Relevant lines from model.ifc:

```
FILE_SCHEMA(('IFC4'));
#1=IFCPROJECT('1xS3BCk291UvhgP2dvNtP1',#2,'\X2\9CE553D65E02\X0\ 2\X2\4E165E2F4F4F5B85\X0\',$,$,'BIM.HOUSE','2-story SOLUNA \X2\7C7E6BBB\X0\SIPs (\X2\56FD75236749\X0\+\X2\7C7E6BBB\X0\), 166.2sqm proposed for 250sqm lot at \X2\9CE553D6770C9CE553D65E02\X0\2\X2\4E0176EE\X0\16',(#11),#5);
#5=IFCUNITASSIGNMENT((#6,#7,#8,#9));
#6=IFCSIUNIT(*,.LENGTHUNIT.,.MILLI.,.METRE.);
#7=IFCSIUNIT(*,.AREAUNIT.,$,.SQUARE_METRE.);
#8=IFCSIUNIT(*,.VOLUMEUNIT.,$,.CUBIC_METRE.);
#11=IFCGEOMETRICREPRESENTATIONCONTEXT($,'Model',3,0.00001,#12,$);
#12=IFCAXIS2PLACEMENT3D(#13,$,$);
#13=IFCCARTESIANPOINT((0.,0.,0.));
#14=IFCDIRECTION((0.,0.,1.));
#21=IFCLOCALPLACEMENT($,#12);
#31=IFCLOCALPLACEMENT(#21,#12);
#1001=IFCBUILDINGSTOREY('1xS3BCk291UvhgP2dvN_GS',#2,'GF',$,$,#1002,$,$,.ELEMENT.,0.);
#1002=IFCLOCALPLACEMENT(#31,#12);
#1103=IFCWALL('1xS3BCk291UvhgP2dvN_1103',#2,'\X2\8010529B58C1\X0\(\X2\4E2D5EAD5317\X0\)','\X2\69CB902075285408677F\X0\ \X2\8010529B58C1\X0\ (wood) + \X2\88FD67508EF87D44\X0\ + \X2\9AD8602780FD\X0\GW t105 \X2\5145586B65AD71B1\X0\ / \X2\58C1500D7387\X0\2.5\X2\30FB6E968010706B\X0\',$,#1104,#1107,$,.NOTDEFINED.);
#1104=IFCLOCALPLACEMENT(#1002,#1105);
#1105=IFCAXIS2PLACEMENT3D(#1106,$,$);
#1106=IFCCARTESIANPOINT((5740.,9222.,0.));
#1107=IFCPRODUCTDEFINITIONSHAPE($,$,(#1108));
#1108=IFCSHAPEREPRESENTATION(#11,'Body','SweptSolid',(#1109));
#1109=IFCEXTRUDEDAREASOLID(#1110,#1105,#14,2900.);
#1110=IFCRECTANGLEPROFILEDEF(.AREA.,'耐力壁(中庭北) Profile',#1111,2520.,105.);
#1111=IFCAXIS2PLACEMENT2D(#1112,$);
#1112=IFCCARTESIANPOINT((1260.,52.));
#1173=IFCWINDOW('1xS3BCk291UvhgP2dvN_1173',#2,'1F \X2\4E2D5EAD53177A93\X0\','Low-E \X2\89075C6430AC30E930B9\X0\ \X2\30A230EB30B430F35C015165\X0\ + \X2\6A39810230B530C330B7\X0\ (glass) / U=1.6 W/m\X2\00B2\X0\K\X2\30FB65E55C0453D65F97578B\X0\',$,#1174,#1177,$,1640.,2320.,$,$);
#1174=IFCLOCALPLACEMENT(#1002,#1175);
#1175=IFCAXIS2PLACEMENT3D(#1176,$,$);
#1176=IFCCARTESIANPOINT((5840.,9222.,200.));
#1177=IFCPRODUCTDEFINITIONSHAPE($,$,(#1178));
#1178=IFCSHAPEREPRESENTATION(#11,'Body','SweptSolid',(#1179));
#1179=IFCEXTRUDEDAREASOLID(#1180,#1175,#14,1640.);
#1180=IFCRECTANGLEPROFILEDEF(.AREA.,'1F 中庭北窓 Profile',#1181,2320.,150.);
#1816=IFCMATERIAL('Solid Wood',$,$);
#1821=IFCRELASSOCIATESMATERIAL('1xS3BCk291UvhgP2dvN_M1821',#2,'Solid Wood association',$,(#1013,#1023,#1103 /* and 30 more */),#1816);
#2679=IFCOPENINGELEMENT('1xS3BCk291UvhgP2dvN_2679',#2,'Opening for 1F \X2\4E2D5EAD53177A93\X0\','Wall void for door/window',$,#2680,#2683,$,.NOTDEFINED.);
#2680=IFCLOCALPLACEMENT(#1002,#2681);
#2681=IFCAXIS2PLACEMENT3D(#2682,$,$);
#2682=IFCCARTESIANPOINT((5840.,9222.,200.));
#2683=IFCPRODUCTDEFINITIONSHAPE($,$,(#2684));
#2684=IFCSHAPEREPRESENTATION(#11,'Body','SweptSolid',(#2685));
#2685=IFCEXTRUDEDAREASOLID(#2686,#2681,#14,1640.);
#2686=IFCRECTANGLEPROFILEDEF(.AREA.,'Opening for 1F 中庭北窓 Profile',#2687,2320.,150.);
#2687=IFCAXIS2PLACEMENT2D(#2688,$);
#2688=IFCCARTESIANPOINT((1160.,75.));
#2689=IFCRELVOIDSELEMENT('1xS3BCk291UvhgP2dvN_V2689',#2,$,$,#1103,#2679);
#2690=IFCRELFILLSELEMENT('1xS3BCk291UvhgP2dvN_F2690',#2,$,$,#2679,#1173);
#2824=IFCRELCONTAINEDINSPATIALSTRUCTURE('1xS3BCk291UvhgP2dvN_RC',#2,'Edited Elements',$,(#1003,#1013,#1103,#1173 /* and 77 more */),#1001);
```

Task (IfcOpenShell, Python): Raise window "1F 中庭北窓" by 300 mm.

```python
import numpy as np
import ifcopenshell
import ifcopenshell.api.geometry
import ifcopenshell.util.placement
import ifcopenshell.util.unit

model = ifcopenshell.open("model.ifc")
unit_scale = ifcopenshell.util.unit.calculate_unit_scale(model)

window = model.by_guid("1xS3BCk291UvhgP2dvN_1173")
opening = window.FillsVoids[0].RelatingOpeningElement
dz = 300.0

shift = np.array([0.0, 0.0, dz])
# The window is not placed relative to its opening, so move both.
for product in (opening, window):
    matrix = ifcopenshell.util.placement.get_local_placement(product.ObjectPlacement)
    matrix[:3, 3] += shift
    ifcopenshell.api.geometry.edit_object_placement(model, product=product, matrix=matrix, is_si=False)

print(f"moved by {dz * unit_scale:+.3f} m")

model.write("model_edited.ifc")
```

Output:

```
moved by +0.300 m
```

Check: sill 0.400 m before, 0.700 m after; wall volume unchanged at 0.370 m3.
